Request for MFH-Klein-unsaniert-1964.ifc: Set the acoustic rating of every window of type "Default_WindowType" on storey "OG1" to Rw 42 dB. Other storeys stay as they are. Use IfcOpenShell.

First a look at what the model holds.

```python
import ifcopenshell
import ifcopenshell.util.element

model = ifcopenshell.open("MFH-Klein-unsaniert-1964.ifc")
print(model.schema)
storey = next(s for s in model.by_type("IfcBuildingStorey") if s.Name == "OG1")
windows = [e for e in ifcopenshell.util.element.get_decomposition(storey) if e.is_a("IfcWindow")]
seen = {}
for e in windows:
    element_type = ifcopenshell.util.element.get_type(e)
    key = (element_type.Name if element_type != e and element_type else None, ifcopenshell.util.element.get_pset(e, "Pset_WindowCommon", "AcousticRating"))
    seen[key] = seen.get(key, 0) + 1
for (name, value), count in sorted(seen.items(), key=str):
    print(count, "x", name, "|", value)
```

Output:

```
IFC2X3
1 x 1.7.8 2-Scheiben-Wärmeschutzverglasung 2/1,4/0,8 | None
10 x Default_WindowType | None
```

```python
import ifcopenshell
import ifcopenshell.api.pset
import ifcopenshell.util.element

model = ifcopenshell.open("MFH-Klein-unsaniert-1964.ifc")

storey = next(s for s in model.by_type("IfcBuildingStorey") if s.Name == "OG1")
windows = [e for e in ifcopenshell.util.element.get_decomposition(storey) if e.is_a("IfcWindow")]

count = 0
for e in windows:
    element_type = ifcopenshell.util.element.get_type(e)
    if element_type in (None, e) or element_type.Name != "Default_WindowType":
        continue
    # add_pset returns the element's existing set when there is one.
    pset = ifcopenshell.api.pset.add_pset(model, product=e, name="Pset_WindowCommon")
    ifcopenshell.api.pset.edit_pset(model, pset=pset, properties={"AcousticRating": "Rw 42 dB"})
    count += 1

print(count, "windows updated")

model.write("MFH-Klein-unsaniert-1964_rev.ifc")
```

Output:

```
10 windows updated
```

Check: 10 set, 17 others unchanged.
